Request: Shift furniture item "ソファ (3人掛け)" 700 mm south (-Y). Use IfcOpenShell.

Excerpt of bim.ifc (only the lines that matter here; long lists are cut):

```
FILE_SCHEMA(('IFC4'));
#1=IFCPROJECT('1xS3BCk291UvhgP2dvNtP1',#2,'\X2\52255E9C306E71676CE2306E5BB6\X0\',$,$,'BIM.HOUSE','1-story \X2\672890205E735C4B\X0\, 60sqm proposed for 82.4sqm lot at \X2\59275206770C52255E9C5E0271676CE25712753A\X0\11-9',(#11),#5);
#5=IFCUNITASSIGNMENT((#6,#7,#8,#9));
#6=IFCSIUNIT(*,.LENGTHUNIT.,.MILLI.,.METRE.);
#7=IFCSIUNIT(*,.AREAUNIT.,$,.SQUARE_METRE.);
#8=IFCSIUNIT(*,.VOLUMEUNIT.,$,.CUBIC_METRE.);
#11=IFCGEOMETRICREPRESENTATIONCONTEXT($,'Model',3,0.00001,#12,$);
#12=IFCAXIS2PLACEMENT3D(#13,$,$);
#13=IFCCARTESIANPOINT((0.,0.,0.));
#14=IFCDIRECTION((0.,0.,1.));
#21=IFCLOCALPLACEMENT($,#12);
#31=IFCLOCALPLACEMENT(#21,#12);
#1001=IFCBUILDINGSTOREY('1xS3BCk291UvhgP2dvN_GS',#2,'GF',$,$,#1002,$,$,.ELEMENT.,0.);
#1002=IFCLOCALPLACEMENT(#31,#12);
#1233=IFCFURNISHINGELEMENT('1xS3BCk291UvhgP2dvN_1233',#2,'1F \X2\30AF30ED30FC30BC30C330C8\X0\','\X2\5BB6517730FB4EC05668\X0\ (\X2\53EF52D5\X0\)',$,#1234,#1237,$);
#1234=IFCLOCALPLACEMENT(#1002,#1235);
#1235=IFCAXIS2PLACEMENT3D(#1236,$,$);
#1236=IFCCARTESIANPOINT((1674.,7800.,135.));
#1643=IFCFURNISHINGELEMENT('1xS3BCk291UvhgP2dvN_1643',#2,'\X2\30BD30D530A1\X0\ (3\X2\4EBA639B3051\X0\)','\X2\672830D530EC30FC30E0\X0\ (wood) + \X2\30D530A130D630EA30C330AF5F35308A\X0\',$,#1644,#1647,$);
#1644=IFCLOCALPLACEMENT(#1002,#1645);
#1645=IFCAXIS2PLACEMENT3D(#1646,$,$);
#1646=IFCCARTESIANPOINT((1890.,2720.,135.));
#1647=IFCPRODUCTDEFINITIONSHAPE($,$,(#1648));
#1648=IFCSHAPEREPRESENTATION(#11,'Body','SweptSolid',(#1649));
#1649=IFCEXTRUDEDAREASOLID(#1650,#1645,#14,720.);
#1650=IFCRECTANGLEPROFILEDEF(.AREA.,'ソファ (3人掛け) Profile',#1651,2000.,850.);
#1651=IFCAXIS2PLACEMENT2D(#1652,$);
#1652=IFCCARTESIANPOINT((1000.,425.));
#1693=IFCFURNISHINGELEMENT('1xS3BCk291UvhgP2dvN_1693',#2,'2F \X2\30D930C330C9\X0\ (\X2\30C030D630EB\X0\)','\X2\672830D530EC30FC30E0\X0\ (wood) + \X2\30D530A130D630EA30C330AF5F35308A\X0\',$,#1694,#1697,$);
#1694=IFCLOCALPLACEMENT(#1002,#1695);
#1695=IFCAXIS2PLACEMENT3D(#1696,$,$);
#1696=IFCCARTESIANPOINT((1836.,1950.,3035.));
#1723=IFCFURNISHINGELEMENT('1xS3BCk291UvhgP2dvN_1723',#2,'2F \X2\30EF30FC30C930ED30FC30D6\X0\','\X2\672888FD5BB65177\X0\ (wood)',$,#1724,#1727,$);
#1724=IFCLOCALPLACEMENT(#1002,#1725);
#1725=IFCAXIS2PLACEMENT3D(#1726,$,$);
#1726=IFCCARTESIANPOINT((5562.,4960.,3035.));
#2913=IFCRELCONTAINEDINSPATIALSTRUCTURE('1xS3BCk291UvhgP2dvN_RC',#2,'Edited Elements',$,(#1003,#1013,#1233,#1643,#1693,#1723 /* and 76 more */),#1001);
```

```python
import ifcopenshell
import ifcopenshell.api.geometry
import ifcopenshell.util.placement
import ifcopenshell.util.unit

model = ifcopenshell.open("bim.ifc")
unit_scale = ifcopenshell.util.unit.calculate_unit_scale(model)

item = model.by_id(1643)
matrix = ifcopenshell.util.placement.get_local_placement(item.ObjectPlacement)
matrix[1, 3] -= 0.7 / unit_scale
ifcopenshell.api.geometry.edit_object_placement(model, product=item, matrix=matrix, is_si=False)

print(ifcopenshell.util.placement.get_local_placement(item.ObjectPlacement).round(3) + 0.0)

model.write("bim_edited.ifc")
```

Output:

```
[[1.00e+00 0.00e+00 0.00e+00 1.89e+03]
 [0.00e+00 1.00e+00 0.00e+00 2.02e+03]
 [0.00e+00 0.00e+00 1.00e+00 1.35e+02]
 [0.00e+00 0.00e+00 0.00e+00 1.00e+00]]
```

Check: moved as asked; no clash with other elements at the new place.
